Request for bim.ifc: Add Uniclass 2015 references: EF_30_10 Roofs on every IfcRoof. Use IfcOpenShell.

First a look at what the model holds.

```python
import ifcopenshell

model = ifcopenshell.open("bim.ifc")
print(model.schema)
print("classifications:", [c.Name for c in model.by_type("IfcClassification")])
for ifc_class in ("IfcDoor", "IfcRoof", "IfcStair", "IfcWall", "IfcWindow"):
    print(ifc_class, len(model.by_type(ifc_class)))
```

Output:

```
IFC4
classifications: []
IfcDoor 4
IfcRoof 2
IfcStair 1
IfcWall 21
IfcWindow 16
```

```python
import ifcopenshell
import ifcopenshell.api.classification

model = ifcopenshell.open("bim.ifc")

system = ifcopenshell.api.classification.add_classification(model, classification="Uniclass 2015")

codes = {
    "IfcRoof": ("EF_30_10", "Roofs"),
}
for ifc_class, (code, name) in codes.items():
    products = model.by_type(ifc_class)
    ifcopenshell.api.classification.add_reference(
        model, products=products, classification=system, identification=code, name=name
    )
    print(code, len(products))

model.write("bim_v2.ifc")
```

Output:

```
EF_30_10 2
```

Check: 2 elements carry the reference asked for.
